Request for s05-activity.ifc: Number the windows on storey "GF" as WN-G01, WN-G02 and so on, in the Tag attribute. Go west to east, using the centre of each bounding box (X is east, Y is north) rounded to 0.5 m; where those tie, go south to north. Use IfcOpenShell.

First a look at what the model holds.

```python
import ifcopenshell
import ifcopenshell.util.element
import ifcopenshell.util.placement

model = ifcopenshell.open("s05-activity.ifc")
print(model.schema)
storey = next(s for s in model.by_type("IfcBuildingStorey") if s.Name == "GF")
windows = [e for e in ifcopenshell.util.element.get_decomposition(storey) if e.is_a("IfcWindow")]
for e in sorted(windows, key=lambda e: e.id()):
    origin = ifcopenshell.util.placement.get_local_placement(e.ObjectPlacement)[:3, 3]
    print(e.id(), e.Tag, e.Name, origin.round(2) + 0.0, sep=" | ")
```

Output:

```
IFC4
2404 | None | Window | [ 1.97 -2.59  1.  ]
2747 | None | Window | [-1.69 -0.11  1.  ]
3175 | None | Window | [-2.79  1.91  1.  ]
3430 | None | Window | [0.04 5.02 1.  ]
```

```python
import ifcopenshell
import ifcopenshell.geom
import ifcopenshell.util.element
import ifcopenshell.util.shape

model = ifcopenshell.open("s05-activity.ifc")
settings = ifcopenshell.geom.settings()
settings.set("use-world-coords", True)


def centre(element):
    shape = ifcopenshell.geom.create_shape(settings, element)
    return ifcopenshell.util.shape.get_bbox_centroid(shape.geometry)


storey = next(s for s in model.by_type("IfcBuildingStorey") if s.Name == "GF")
windows = [e for e in ifcopenshell.util.element.get_decomposition(storey) if e.is_a("IfcWindow")]

# Insertion points can sit at a corner or the storey origin, so sort by the geometry (in metres).
centres = {e: centre(e) for e in windows}
windows.sort(key=lambda e: (round(centres[e][0] / 0.5), centres[e][1]))

for i, e in enumerate(windows, start=1):
    number = f"WN-G{i:02d}"
    e.Tag = number
    print(e.id(), number)

model.write("s05-activity_updated.ifc")
```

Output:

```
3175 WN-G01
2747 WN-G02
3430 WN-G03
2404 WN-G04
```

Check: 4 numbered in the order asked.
